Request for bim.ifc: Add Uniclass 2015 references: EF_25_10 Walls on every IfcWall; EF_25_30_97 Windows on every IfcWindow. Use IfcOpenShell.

First a look at what the model holds.

```python
import ifcopenshell

model = ifcopenshell.open("bim.ifc")
print(model.schema)
print("classifications:", [c.Name for c in model.by_type("IfcClassification")])
for ifc_class in ("IfcDoor", "IfcRoof", "IfcStair", "IfcWall", "IfcWindow"):
    print(ifc_class, len(model.by_type(ifc_class)))
```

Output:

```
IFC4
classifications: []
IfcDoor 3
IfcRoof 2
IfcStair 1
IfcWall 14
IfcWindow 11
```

```python
import ifcopenshell
import ifcopenshell.api.classification

model = ifcopenshell.open("bim.ifc")

system = ifcopenshell.api.classification.add_classification(model, classification="Uniclass 2015")

codes = {
    "IfcWall": ("EF_25_10", "Walls"),
    "IfcWindow": ("EF_25_30_97", "Windows"),
}
for ifc_class, (code, name) in codes.items():
    products = model.by_type(ifc_class)
    ifcopenshell.api.classification.add_reference(
        model, products=products, classification=system, identification=code, name=name
    )
    print(code, len(products))

model.write("bim_v2.ifc")
```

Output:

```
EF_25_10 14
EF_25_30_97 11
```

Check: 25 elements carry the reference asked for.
